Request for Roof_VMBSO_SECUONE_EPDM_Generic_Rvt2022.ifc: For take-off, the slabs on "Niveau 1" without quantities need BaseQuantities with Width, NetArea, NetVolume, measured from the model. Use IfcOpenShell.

First a look at what the model holds.

```python
import ifcopenshell
import ifcopenshell.util.element
import ifcopenshell.util.unit

model = ifcopenshell.open("Roof_VMBSO_SECUONE_EPDM_Generic_Rvt2022.ifc")
print(model.schema)
for unit_type in ("LENGTHUNIT", "AREAUNIT", "VOLUMEUNIT"):
    print(unit_type, ifcopenshell.util.unit.calculate_unit_scale(model, unit_type))
storey = next(s for s in model.by_type("IfcBuildingStorey") if s.Name == "Niveau 1")
slabs = [e for e in ifcopenshell.util.element.get_decomposition(storey) if e.is_a("IfcSlab")]
for e in sorted(slabs, key=lambda e: e.id()):
    print(e.id(), e.is_a(), e.Name, list(ifcopenshell.util.element.get_psets(e, qtos_only=True)), sep=" | ")
```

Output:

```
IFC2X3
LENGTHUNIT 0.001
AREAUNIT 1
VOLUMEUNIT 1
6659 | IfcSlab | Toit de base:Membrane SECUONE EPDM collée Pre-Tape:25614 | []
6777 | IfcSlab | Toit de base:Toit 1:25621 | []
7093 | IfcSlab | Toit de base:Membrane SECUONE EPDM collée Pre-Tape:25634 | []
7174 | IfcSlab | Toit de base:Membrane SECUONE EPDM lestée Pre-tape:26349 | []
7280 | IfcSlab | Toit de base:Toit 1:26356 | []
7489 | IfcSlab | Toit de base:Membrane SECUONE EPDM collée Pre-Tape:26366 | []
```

```python
import ifcopenshell
import ifcopenshell.api.pset
import ifcopenshell.geom
import ifcopenshell.util.element
import ifcopenshell.util.shape
import ifcopenshell.util.unit

model = ifcopenshell.open("Roof_VMBSO_SECUONE_EPDM_Generic_Rvt2022.ifc")
unit_scale = ifcopenshell.util.unit.calculate_unit_scale(model)
area_scale = ifcopenshell.util.unit.calculate_unit_scale(model, "AREAUNIT")
volume_scale = ifcopenshell.util.unit.calculate_unit_scale(model, "VOLUMEUNIT")
settings = ifcopenshell.geom.settings()

storey = next(s for s in model.by_type("IfcBuildingStorey") if s.Name == "Niveau 1")
slabs = [e for e in ifcopenshell.util.element.get_decomposition(storey) if e.is_a("IfcSlab")]

for e in sorted(slabs, key=lambda e: e.id()):
    if ifcopenshell.util.element.get_psets(e, qtos_only=True, should_inherit=False):
        continue
    # Geometry comes back in metres, in the element's own axes.
    shape = ifcopenshell.geom.create_shape(settings, e)
    values = {
        "Width": ifcopenshell.util.shape.get_z(shape.geometry) / unit_scale,
        "NetArea": ifcopenshell.util.shape.get_footprint_area(shape.geometry) / area_scale,
        "NetVolume": ifcopenshell.util.shape.get_volume(shape.geometry) / volume_scale,
    }
    qto = ifcopenshell.api.pset.add_qto(model, product=e, name="BaseQuantities")
    ifcopenshell.api.pset.edit_qto(model, qto=qto, properties=values)
    print(e.id(), {k: round(v, 3) for k, v in values.items()})

model.write("Roof_VMBSO_SECUONE_EPDM_Generic_Rvt2022_v2.ifc")
```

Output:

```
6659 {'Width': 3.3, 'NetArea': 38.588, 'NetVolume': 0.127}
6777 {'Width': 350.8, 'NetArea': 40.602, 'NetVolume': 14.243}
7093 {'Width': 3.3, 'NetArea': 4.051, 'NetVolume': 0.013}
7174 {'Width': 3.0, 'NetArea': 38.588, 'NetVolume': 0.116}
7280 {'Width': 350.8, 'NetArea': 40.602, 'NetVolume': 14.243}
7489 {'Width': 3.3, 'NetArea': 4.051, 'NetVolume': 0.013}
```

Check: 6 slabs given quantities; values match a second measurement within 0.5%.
